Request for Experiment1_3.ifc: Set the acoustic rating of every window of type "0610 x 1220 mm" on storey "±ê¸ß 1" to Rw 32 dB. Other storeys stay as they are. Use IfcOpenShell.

First a look at what the model holds.

```python
import ifcopenshell
import ifcopenshell.util.element

model = ifcopenshell.open("Experiment1_3.ifc")
print(model.schema)
storey = next(s for s in model.by_type("IfcBuildingStorey") if s.Name == "±ê¸ß 1")
windows = [e for e in ifcopenshell.util.element.get_decomposition(storey) if e.is_a("IfcWindow")]
seen = {}
for e in windows:
    element_type = ifcopenshell.util.element.get_type(e)
    key = (element_type.Name if element_type != e and element_type else None, ifcopenshell.util.element.get_pset(e, "Pset_WindowCommon", "AcousticRating"))
    seen[key] = seen.get(key, 0) + 1
for (name, value), count in sorted(seen.items(), key=str):
    print(count, "x", name, "|", value)
```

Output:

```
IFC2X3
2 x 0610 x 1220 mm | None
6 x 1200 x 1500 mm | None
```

```python
import ifcopenshell
import ifcopenshell.api.pset
import ifcopenshell.util.element

model = ifcopenshell.open("Experiment1_3.ifc")

storey = next(s for s in model.by_type("IfcBuildingStorey") if s.Name == "±ê¸ß 1")
windows = [e for e in ifcopenshell.util.element.get_decomposition(storey) if e.is_a("IfcWindow")]

count = 0
for e in windows:
    element_type = ifcopenshell.util.element.get_type(e)
    if element_type in (None, e) or element_type.Name != "0610 x 1220 mm":
        continue
    # add_pset returns the element's existing set when there is one.
    pset = ifcopenshell.api.pset.add_pset(model, product=e, name="Pset_WindowCommon")
    ifcopenshell.api.pset.edit_pset(model, pset=pset, properties={"AcousticRating": "Rw 32 dB"})
    count += 1

print(count, "windows updated")

model.write("Experiment1_3_updated.ifc")
```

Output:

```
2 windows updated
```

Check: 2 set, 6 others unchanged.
